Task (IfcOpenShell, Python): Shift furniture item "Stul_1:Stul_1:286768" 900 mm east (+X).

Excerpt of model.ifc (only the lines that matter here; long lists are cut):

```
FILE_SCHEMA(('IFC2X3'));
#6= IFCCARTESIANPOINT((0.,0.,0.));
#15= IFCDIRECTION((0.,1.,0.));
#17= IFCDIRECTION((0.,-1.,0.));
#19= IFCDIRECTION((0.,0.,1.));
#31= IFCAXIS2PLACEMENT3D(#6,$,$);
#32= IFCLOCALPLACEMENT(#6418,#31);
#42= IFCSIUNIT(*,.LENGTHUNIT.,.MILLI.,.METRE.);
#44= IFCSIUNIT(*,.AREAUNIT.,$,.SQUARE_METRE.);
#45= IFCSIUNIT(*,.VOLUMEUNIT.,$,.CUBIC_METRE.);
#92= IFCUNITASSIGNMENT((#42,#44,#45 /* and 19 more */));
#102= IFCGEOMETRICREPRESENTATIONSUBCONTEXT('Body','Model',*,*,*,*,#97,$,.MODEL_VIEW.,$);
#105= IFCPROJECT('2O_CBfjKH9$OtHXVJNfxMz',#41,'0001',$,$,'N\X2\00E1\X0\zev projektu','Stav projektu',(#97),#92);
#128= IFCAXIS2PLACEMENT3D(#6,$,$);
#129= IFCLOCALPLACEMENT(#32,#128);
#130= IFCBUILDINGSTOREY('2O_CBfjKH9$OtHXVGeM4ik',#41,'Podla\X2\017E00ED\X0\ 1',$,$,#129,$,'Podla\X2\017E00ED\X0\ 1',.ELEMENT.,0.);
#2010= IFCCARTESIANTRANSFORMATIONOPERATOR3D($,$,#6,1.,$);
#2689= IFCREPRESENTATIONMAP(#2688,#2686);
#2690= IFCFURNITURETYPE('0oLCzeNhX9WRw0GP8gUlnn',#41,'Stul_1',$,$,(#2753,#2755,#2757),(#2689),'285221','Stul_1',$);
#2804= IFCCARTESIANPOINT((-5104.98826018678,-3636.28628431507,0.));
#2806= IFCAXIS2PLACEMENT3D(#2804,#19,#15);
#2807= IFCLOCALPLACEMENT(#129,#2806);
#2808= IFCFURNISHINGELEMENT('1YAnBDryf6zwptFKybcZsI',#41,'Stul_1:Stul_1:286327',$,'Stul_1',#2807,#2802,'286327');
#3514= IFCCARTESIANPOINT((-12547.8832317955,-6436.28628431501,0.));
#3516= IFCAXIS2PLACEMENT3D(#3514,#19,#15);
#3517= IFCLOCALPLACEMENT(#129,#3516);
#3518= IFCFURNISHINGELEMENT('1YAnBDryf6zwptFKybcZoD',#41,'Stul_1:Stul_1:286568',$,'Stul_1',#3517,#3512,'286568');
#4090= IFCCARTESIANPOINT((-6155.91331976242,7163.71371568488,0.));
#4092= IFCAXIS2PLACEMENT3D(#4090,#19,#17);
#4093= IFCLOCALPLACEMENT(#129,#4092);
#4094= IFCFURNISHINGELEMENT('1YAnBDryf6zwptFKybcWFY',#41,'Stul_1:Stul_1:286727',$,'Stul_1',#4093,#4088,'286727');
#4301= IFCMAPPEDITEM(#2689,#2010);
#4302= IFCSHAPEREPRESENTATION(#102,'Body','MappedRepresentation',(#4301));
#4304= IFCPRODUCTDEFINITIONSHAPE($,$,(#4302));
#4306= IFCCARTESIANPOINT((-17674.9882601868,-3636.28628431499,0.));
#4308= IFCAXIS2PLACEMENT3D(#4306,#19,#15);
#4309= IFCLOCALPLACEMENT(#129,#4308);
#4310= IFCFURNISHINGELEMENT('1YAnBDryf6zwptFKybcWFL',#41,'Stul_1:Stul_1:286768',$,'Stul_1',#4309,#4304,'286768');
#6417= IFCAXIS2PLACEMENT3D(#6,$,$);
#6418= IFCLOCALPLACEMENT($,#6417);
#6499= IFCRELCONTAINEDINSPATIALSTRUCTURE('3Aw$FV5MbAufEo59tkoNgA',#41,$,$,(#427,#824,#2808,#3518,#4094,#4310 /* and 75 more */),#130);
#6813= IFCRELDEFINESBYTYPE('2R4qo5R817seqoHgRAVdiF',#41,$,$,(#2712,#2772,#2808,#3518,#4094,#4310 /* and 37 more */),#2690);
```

```python
import ifcopenshell
import ifcopenshell.api.geometry
import ifcopenshell.util.placement
import ifcopenshell.util.unit

model = ifcopenshell.open("model.ifc")
unit_scale = ifcopenshell.util.unit.calculate_unit_scale(model)

item = model.by_guid("1YAnBDryf6zwptFKybcWFL")
matrix = ifcopenshell.util.placement.get_local_placement(item.ObjectPlacement)
matrix[0, 3] += 0.9 / unit_scale
ifcopenshell.api.geometry.edit_object_placement(model, product=item, matrix=matrix, is_si=False)

print(ifcopenshell.util.placement.get_local_placement(item.ObjectPlacement).round(3) + 0.0)

model.write("model-out.ifc")
```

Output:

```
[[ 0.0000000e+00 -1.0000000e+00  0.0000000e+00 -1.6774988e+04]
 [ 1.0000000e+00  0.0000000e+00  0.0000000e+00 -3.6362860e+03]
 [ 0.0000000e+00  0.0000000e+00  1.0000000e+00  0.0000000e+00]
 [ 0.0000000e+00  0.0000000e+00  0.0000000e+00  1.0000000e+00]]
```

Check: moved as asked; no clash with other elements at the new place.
